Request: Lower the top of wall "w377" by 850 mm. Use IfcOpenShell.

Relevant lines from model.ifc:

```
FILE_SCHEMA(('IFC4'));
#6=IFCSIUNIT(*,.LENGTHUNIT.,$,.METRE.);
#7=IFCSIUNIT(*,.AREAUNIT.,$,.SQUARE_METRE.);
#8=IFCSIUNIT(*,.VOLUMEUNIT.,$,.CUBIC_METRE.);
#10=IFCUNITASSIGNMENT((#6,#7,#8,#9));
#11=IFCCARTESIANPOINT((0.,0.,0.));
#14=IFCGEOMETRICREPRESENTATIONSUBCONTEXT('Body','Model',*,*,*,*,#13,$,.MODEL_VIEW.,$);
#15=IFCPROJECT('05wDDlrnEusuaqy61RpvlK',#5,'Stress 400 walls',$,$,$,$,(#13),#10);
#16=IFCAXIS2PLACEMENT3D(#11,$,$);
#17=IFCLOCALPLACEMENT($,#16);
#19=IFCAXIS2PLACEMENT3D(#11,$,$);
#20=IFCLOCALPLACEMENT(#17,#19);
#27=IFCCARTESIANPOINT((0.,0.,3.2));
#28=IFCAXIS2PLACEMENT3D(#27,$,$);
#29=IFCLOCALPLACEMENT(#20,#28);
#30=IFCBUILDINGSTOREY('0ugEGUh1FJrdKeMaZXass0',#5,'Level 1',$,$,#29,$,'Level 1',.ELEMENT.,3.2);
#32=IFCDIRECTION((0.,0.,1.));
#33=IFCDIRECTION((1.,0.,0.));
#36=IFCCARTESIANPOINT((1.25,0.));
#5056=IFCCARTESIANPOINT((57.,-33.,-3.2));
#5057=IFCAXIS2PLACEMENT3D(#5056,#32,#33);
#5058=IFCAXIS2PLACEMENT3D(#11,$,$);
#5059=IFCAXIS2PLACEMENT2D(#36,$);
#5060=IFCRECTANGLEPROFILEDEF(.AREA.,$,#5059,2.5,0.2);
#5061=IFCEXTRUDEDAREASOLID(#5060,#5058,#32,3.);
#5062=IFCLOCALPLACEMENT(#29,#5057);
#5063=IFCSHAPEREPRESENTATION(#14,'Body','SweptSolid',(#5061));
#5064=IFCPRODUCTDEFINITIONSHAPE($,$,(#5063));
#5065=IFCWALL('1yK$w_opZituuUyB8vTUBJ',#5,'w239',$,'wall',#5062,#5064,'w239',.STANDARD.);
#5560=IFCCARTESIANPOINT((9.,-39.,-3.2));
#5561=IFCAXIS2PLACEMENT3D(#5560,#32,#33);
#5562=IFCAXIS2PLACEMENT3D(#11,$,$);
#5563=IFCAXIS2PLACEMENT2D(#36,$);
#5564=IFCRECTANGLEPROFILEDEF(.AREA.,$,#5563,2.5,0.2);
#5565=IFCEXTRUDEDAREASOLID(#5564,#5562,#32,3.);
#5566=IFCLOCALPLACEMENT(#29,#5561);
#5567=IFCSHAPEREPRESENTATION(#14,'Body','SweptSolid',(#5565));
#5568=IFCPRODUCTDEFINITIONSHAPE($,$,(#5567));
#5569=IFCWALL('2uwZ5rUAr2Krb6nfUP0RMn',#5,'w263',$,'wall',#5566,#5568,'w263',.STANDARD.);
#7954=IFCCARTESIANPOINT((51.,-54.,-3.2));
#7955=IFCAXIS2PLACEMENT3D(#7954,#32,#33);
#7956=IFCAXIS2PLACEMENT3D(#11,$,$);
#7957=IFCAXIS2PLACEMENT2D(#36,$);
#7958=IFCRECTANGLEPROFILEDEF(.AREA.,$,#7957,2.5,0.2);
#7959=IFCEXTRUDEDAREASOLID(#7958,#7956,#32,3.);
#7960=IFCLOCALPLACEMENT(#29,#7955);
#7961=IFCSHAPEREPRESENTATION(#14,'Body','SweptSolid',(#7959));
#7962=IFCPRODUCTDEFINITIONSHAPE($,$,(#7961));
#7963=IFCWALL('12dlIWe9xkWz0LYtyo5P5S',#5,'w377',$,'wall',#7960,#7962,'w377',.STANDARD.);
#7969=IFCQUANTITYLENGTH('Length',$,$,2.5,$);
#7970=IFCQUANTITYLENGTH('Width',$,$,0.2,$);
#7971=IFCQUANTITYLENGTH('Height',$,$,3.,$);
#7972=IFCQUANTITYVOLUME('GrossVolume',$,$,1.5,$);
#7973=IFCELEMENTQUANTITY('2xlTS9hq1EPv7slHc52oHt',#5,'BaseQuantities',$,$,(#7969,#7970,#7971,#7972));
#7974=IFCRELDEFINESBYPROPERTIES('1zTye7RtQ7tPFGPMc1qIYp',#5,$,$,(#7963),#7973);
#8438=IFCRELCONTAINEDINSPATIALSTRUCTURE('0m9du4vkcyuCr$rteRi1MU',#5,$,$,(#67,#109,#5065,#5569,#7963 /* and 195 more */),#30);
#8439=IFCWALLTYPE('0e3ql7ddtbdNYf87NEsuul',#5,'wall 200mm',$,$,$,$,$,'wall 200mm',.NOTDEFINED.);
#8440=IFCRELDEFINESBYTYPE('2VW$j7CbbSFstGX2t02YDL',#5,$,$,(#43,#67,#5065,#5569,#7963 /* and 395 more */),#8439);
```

```python
import ifcopenshell
import ifcopenshell.api.pset
import ifcopenshell.geom
import ifcopenshell.util.element
import ifcopenshell.util.representation
import ifcopenshell.util.shape
import ifcopenshell.util.unit

model = ifcopenshell.open("model.ifc")
unit_scale = ifcopenshell.util.unit.calculate_unit_scale(model)
volume_scale = ifcopenshell.util.unit.calculate_unit_scale(model, "VOLUMEUNIT")
settings = ifcopenshell.geom.settings()


def volume(element):
    """Net volume in cubic metres, openings subtracted."""
    shape = ifcopenshell.geom.create_shape(settings, element)
    return ifcopenshell.util.shape.get_volume(shape.geometry)


wall = model.by_guid("12dlIWe9xkWz0LYtyo5P5S")
before = volume(wall)

body = ifcopenshell.util.representation.get_representation(wall, "Model", "Body")
solid = body.Items[0]
old_height = solid.Depth
solid.Depth -= 0.85 / unit_scale
after = volume(wall)

# Update the stored height, areas and volumes.
qto = model.by_id(ifcopenshell.util.element.get_pset(wall, "BaseQuantities", should_inherit=False)["id"])
ifcopenshell.api.pset.edit_qto(model, qto=qto, properties={
    "Height": solid.Depth,
    "GrossVolume": ifcopenshell.util.element.get_pset(wall, "BaseQuantities", "GrossVolume") * solid.Depth / old_height,
})

print(f"height {old_height:g} -> {solid.Depth:g}, volume {before:.3f} -> {after:.3f} m3")

model.write("model_rev.ifc")
```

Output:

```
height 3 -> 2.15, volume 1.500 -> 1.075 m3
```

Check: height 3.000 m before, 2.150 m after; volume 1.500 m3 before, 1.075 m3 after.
